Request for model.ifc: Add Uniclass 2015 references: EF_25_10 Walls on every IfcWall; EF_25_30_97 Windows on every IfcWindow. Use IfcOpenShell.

First a look at what the model holds.

```python
import ifcopenshell

model = ifcopenshell.open("model.ifc")
print(model.schema)
print("classifications:", [c.Name for c in model.by_type("IfcClassification")])
for ifc_class in ("IfcDoor", "IfcRoof", "IfcStair", "IfcWall", "IfcWindow"):
    print(ifc_class, len(model.by_type(ifc_class)))
```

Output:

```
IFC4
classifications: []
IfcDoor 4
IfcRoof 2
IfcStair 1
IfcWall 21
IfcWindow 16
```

```python
import ifcopenshell
import ifcopenshell.api.classification

model = ifcopenshell.open("model.ifc")

system = ifcopenshell.api.classification.add_classification(model, classification="Uniclass 2015")

codes = {
    "IfcWall": ("EF_25_10", "Walls"),
    "IfcWindow": ("EF_25_30_97", "Windows"),
}
for ifc_class, (code, name) in codes.items():
    products = model.by_type(ifc_class)
    ifcopenshell.api.classification.add_reference(
        model, products=products, classification=system, identification=code, name=name
    )
    print(code, len(products))

model.write("model_edited.ifc")
```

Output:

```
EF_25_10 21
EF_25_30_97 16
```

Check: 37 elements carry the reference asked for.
